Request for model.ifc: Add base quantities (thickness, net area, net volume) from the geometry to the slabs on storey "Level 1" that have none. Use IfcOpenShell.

First a look at what the model holds.

```python
import ifcopenshell
import ifcopenshell.util.element
import ifcopenshell.util.unit

model = ifcopenshell.open("model.ifc")
print(model.schema)
for unit_type in ("LENGTHUNIT", "AREAUNIT", "VOLUMEUNIT"):
    print(unit_type, ifcopenshell.util.unit.calculate_unit_scale(model, unit_type))
storey = next(s for s in model.by_type("IfcBuildingStorey") if s.Name == "Level 1")
slabs = [e for e in ifcopenshell.util.element.get_decomposition(storey) if e.is_a("IfcSlab")]
for e in sorted(slabs, key=lambda e: e.id()):
    print(e.id(), e.is_a(), e.Name, list(ifcopenshell.util.element.get_psets(e, qtos_only=True)), sep=" | ")
```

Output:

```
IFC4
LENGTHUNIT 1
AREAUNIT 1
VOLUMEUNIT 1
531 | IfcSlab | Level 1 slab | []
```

```python
import ifcopenshell
import ifcopenshell.api.pset
import ifcopenshell.geom
import ifcopenshell.util.element
import ifcopenshell.util.shape
import ifcopenshell.util.unit

model = ifcopenshell.open("model.ifc")
unit_scale = ifcopenshell.util.unit.calculate_unit_scale(model)
area_scale = ifcopenshell.util.unit.calculate_unit_scale(model, "AREAUNIT")
volume_scale = ifcopenshell.util.unit.calculate_unit_scale(model, "VOLUMEUNIT")
settings = ifcopenshell.geom.settings()

storey = next(s for s in model.by_type("IfcBuildingStorey") if s.Name == "Level 1")
slabs = [e for e in ifcopenshell.util.element.get_decomposition(storey) if e.is_a("IfcSlab")]

for e in sorted(slabs, key=lambda e: e.id()):
    if ifcopenshell.util.element.get_psets(e, qtos_only=True, should_inherit=False):
        continue
    # Geometry comes back in metres, in the element's own axes.
    shape = ifcopenshell.geom.create_shape(settings, e)
    values = {
        "Width": ifcopenshell.util.shape.get_z(shape.geometry) / unit_scale,
        "NetArea": ifcopenshell.util.shape.get_footprint_area(shape.geometry) / area_scale,
        "NetVolume": ifcopenshell.util.shape.get_volume(shape.geometry) / volume_scale,
    }
    qto = ifcopenshell.api.pset.add_qto(model, product=e, name="Qto_SlabBaseQuantities")
    ifcopenshell.api.pset.edit_qto(model, qto=qto, properties=values)
    print(e.id(), {k: round(v, 3) for k, v in values.items()})

model.write("model_v2.ifc")
```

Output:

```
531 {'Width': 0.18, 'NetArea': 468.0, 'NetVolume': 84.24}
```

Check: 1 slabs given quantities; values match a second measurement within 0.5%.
